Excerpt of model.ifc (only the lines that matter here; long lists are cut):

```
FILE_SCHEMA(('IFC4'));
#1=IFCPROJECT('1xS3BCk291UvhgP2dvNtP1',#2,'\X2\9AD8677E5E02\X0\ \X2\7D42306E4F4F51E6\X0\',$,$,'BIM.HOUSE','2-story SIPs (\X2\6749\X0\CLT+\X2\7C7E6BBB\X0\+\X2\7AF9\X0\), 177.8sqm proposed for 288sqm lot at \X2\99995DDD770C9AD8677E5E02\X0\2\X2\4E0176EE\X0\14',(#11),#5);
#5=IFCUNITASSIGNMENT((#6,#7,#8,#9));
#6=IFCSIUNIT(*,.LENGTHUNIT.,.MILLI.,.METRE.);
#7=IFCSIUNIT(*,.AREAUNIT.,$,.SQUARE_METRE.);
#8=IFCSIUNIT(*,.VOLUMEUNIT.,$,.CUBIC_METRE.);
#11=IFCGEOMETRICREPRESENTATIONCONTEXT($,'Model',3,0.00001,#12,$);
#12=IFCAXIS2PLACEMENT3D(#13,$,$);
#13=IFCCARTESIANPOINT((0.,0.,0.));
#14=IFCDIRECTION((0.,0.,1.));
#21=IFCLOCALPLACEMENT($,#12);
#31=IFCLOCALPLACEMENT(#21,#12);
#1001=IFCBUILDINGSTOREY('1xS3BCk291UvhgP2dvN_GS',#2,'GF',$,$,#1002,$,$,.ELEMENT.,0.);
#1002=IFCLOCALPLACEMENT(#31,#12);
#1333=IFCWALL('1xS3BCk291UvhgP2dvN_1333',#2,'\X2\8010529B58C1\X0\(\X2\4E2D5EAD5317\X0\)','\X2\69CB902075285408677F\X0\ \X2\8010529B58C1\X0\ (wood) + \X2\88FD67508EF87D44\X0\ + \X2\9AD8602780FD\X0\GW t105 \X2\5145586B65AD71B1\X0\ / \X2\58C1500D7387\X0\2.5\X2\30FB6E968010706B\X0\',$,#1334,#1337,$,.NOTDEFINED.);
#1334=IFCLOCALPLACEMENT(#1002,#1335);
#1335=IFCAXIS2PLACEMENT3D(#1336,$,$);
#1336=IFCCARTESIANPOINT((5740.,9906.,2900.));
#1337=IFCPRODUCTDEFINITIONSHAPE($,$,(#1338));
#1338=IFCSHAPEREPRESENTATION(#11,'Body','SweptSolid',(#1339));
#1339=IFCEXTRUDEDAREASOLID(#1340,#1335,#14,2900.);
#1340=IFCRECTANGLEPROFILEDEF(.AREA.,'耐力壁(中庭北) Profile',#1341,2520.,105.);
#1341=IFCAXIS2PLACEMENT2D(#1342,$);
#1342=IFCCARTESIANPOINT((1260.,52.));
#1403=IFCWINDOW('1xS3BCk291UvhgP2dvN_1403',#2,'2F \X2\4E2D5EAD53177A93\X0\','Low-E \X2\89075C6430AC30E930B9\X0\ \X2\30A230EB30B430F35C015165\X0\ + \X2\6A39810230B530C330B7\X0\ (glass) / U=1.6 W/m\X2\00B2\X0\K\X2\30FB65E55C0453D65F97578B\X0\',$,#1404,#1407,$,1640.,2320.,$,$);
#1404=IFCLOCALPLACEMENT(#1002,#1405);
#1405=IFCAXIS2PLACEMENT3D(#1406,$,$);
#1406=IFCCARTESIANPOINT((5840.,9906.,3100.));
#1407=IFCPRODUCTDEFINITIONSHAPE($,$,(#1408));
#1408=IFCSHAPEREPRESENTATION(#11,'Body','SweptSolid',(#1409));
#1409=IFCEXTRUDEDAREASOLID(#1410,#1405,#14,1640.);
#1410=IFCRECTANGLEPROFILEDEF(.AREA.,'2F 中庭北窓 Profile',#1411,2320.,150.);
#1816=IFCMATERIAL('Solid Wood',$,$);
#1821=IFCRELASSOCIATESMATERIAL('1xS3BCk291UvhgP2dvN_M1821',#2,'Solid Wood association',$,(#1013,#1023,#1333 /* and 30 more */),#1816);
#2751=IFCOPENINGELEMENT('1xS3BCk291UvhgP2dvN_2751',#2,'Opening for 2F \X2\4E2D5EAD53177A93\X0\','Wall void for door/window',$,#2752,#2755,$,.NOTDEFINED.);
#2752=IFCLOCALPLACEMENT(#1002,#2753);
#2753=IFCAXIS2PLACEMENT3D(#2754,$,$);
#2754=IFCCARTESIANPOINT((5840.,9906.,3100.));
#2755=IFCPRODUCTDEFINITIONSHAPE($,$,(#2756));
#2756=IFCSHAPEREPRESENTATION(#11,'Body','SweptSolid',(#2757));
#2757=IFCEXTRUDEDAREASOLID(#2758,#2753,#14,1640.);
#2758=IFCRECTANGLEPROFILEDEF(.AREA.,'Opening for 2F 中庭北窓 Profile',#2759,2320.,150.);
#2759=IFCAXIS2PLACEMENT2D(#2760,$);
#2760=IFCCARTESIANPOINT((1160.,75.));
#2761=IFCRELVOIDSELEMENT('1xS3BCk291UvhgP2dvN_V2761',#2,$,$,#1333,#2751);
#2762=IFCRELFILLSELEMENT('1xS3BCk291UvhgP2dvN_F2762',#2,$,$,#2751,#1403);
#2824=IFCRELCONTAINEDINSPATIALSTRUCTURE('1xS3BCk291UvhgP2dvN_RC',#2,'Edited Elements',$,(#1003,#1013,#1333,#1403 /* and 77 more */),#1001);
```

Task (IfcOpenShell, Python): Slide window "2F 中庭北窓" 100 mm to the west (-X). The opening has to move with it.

```python
import ifcopenshell
import ifcopenshell.api.geometry
import ifcopenshell.util.placement
import ifcopenshell.util.unit

model = ifcopenshell.open("model.ifc")
unit_scale = ifcopenshell.util.unit.calculate_unit_scale(model)

window = model.by_id(1403)
opening = window.FillsVoids[0].RelatingOpeningElement
wall = opening.VoidsElements[0].RelatingBuildingElement

wall_matrix = ifcopenshell.util.placement.get_local_placement(wall.ObjectPlacement)
shift = wall_matrix[:3, 0] * -0.1 / unit_scale
before = ifcopenshell.util.placement.get_local_placement(window.ObjectPlacement)[:3, 3].copy()

# The window is not placed relative to its opening, so move both.
for product in (opening, window):
    matrix = ifcopenshell.util.placement.get_local_placement(product.ObjectPlacement)
    matrix[:3, 3] += shift
    ifcopenshell.api.geometry.edit_object_placement(model, product=product, matrix=matrix, is_si=False)

after = ifcopenshell.util.placement.get_local_placement(window.ObjectPlacement)[:3, 3]
print("window moved by", (after - before).round(3) + 0.0)

model.write("model_rev.ifc")
```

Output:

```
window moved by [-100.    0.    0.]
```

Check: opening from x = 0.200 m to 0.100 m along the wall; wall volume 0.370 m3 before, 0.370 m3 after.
